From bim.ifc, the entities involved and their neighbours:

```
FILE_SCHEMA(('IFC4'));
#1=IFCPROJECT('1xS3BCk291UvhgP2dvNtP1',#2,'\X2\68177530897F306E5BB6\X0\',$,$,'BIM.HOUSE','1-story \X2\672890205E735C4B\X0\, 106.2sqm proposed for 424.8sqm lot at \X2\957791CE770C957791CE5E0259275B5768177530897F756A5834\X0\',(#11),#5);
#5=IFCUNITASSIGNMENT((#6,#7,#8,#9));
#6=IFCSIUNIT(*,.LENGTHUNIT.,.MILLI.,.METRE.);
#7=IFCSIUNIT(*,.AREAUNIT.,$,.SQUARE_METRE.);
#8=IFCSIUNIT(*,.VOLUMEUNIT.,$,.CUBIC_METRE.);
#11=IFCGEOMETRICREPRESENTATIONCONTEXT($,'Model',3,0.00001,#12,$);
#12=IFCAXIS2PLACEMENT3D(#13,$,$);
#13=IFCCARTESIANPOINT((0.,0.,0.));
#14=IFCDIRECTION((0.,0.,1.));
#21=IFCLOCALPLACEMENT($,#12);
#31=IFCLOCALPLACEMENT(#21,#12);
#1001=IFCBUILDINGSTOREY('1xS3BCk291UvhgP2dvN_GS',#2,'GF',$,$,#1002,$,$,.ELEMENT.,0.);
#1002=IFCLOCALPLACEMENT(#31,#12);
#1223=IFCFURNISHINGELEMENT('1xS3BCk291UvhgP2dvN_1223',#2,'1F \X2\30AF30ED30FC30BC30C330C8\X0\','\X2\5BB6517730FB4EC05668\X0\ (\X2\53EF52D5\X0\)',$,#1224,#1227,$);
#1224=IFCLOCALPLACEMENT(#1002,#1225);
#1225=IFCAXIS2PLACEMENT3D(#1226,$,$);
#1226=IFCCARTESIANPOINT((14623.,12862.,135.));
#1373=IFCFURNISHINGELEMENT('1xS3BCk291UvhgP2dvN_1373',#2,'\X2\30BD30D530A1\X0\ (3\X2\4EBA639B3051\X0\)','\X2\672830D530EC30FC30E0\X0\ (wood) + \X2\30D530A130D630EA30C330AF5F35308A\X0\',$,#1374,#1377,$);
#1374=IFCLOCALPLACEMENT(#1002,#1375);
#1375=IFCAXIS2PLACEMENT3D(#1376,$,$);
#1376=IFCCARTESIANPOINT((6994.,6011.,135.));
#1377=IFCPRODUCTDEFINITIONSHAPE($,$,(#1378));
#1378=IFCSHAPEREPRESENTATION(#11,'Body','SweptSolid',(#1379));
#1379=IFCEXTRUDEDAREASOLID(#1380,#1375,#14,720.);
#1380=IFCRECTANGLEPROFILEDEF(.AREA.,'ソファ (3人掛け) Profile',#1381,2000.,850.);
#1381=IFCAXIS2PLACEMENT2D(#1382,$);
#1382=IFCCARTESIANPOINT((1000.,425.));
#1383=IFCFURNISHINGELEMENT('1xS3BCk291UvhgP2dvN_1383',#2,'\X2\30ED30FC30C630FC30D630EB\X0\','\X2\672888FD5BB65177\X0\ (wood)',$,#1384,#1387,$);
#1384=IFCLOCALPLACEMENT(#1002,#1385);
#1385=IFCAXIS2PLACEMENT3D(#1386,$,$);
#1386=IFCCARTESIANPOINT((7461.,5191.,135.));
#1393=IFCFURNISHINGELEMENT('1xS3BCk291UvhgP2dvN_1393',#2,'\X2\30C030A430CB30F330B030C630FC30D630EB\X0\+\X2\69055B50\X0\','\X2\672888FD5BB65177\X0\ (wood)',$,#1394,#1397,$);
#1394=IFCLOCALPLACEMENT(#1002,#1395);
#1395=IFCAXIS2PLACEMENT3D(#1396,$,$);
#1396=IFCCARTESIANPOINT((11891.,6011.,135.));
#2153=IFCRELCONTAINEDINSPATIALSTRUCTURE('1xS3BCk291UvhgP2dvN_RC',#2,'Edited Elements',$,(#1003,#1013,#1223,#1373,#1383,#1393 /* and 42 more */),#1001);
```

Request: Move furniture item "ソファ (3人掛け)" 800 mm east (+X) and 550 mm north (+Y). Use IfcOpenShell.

```python
import ifcopenshell
import ifcopenshell.api.geometry
import ifcopenshell.util.placement
import ifcopenshell.util.unit

model = ifcopenshell.open("bim.ifc")
unit_scale = ifcopenshell.util.unit.calculate_unit_scale(model)

item = model.by_guid("1xS3BCk291UvhgP2dvN_1373")
matrix = ifcopenshell.util.placement.get_local_placement(item.ObjectPlacement)
matrix[0, 3] += 0.8 / unit_scale
matrix[1, 3] += 0.55 / unit_scale
ifcopenshell.api.geometry.edit_object_placement(model, product=item, matrix=matrix, is_si=False)

print(ifcopenshell.util.placement.get_local_placement(item.ObjectPlacement).round(3) + 0.0)

model.write("bim_edited.ifc")
```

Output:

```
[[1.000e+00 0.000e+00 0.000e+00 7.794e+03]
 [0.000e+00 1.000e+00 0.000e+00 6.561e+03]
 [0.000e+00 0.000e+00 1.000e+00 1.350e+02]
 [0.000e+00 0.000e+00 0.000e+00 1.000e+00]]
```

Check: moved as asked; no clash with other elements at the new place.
